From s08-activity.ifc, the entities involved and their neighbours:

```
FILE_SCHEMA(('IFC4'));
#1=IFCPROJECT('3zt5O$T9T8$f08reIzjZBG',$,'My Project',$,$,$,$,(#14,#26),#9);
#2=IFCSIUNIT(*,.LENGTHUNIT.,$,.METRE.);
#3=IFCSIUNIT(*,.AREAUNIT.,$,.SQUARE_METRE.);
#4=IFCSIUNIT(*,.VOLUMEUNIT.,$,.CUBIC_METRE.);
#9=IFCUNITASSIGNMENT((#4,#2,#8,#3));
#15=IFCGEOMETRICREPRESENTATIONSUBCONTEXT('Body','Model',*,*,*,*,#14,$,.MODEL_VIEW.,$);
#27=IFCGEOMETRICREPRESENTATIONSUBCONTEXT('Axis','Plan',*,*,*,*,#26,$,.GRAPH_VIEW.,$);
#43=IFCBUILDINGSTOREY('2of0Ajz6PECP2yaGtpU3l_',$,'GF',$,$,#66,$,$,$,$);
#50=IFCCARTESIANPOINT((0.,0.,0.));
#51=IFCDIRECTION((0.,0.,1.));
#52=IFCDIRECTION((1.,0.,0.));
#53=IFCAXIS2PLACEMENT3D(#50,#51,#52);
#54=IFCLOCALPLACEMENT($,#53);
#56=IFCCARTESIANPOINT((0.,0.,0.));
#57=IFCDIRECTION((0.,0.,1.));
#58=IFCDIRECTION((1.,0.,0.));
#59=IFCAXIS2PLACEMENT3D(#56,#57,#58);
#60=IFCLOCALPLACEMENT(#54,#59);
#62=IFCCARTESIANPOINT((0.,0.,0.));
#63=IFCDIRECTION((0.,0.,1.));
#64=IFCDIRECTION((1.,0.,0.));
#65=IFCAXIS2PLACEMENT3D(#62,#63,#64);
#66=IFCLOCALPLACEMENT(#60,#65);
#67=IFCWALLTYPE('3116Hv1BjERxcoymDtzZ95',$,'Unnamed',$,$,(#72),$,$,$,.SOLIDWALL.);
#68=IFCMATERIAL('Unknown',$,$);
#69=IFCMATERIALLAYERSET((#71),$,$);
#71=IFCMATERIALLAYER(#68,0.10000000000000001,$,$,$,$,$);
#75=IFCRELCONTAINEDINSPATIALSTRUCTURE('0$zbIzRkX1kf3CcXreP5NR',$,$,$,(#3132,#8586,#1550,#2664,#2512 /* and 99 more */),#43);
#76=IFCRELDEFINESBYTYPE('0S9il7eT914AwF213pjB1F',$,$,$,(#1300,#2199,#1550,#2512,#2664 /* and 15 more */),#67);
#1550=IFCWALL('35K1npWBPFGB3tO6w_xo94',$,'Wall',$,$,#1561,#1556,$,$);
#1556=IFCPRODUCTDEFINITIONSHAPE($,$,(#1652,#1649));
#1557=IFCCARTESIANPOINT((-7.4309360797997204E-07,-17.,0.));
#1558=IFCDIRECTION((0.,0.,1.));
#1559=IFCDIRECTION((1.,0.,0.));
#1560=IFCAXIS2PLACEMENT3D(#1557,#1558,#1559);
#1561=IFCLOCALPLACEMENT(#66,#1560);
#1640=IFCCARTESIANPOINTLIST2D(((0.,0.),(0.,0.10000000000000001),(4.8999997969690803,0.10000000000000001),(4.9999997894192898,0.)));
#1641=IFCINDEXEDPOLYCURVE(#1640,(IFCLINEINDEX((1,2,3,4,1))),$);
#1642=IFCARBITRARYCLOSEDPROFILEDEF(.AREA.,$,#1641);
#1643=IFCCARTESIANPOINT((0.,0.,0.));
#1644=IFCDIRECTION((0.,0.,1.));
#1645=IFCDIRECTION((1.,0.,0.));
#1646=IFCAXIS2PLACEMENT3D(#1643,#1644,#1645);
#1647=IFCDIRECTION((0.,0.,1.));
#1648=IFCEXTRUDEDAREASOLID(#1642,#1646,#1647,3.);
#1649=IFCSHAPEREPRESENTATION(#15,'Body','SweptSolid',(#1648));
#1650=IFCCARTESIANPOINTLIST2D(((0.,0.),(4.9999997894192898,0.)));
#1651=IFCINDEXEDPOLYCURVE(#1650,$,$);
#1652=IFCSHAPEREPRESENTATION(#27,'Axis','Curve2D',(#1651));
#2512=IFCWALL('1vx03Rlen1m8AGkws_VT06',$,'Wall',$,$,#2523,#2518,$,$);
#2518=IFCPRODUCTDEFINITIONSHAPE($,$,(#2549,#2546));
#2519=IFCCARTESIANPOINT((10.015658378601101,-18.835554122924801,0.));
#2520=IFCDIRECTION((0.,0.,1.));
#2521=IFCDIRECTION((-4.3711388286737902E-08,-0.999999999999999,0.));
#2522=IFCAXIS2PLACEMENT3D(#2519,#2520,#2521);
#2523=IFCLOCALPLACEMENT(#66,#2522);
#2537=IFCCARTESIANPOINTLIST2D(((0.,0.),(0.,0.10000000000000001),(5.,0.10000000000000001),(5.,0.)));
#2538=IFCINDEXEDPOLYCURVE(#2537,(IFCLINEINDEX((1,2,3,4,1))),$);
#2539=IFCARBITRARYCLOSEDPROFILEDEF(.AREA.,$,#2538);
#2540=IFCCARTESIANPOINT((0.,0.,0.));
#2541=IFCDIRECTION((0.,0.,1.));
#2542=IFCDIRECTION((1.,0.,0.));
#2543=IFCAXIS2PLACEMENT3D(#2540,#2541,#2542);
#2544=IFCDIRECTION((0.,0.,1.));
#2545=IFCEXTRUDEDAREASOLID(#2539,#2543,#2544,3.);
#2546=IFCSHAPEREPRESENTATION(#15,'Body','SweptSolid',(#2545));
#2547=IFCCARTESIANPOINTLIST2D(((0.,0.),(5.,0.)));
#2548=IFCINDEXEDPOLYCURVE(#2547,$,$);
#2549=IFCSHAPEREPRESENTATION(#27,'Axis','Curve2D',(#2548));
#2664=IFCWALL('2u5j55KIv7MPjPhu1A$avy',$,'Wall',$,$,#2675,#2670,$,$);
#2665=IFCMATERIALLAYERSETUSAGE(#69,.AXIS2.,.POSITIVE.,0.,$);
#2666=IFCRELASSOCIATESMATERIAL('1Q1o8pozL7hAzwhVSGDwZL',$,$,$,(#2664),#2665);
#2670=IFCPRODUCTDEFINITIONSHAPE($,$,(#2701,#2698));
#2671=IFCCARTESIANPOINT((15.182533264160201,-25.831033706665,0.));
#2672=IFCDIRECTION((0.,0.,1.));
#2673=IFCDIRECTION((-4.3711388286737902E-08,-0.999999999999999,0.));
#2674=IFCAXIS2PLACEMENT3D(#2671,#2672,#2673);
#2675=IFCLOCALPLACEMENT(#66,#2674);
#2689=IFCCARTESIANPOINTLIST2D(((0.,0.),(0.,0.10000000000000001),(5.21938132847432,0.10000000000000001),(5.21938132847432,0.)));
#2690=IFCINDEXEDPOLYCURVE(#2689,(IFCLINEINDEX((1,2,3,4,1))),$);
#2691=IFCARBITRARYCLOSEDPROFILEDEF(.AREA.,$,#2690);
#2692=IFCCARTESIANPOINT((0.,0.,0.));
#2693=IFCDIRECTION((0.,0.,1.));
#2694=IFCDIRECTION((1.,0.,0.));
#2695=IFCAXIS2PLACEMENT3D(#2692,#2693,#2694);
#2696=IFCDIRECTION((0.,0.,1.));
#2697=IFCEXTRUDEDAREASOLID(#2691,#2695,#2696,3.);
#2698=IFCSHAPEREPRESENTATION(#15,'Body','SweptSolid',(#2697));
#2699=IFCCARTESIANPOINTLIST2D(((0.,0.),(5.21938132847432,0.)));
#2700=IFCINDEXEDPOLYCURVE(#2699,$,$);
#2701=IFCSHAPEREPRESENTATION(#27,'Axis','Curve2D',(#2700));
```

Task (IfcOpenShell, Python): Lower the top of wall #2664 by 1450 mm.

```python
import ifcopenshell
import ifcopenshell.geom
import ifcopenshell.util.representation
import ifcopenshell.util.shape
import ifcopenshell.util.unit

model = ifcopenshell.open("s08-activity.ifc")
unit_scale = ifcopenshell.util.unit.calculate_unit_scale(model)
settings = ifcopenshell.geom.settings()


def volume(element):
    """Net volume in cubic metres, openings subtracted."""
    shape = ifcopenshell.geom.create_shape(settings, element)
    return ifcopenshell.util.shape.get_volume(shape.geometry)


wall = model.by_guid("2u5j55KIv7MPjPhu1A$avy")
before = volume(wall)

body = ifcopenshell.util.representation.get_representation(wall, "Model", "Body")
solid = body.Items[0]
old_height = solid.Depth
solid.Depth -= 1.45 / unit_scale
after = volume(wall)

print(f"height {old_height:g} -> {solid.Depth:g}, volume {before:.3f} -> {after:.3f} m3")

model.write("s08-activity_rev.ifc")
```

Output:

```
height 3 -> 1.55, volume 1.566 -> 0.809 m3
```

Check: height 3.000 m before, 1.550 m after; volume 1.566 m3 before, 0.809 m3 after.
